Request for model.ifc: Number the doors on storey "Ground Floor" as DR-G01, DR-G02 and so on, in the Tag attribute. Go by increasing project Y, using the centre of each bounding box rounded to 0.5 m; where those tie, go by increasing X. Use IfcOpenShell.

First a look at what the model holds.

```python
import ifcopenshell
import ifcopenshell.util.element
import ifcopenshell.util.placement

model = ifcopenshell.open("model.ifc")
print(model.schema)
storey = next(s for s in model.by_type("IfcBuildingStorey") if s.Name == "Ground Floor")
doors = [e for e in ifcopenshell.util.element.get_decomposition(storey) if e.is_a("IfcDoor")]
for e in sorted(doors, key=lambda e: e.id()):
    origin = ifcopenshell.util.placement.get_local_placement(e.ObjectPlacement)[:3, 3]
    print(e.id(), e.Tag, e.Name, origin.round(2) + 0.0, sep=" | ")
```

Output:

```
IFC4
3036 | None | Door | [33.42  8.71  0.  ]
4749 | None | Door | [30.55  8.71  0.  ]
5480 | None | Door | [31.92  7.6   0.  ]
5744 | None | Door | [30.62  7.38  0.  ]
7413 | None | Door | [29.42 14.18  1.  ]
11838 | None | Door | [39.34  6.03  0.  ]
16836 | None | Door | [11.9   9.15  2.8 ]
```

```python
import ifcopenshell
import ifcopenshell.geom
import ifcopenshell.util.element
import ifcopenshell.util.shape

model = ifcopenshell.open("model.ifc")
settings = ifcopenshell.geom.settings()
settings.set("use-world-coords", True)


def centre(element):
    shape = ifcopenshell.geom.create_shape(settings, element)
    return ifcopenshell.util.shape.get_bbox_centroid(shape.geometry)


storey = next(s for s in model.by_type("IfcBuildingStorey") if s.Name == "Ground Floor")
doors = [e for e in ifcopenshell.util.element.get_decomposition(storey) if e.is_a("IfcDoor")]

# Insertion points can sit at a corner or the storey origin, so sort by the geometry (in metres).
centres = {e: centre(e) for e in doors}
doors.sort(key=lambda e: (round(centres[e][1] / 0.5), centres[e][0]))

for i, e in enumerate(doors, start=1):
    number = f"DR-G{i:02d}"
    e.Tag = number
    print(e.id(), number)

model.write("model-out.ifc")
```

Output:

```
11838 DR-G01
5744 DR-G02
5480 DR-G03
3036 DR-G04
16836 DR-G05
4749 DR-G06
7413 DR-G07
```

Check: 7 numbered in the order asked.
